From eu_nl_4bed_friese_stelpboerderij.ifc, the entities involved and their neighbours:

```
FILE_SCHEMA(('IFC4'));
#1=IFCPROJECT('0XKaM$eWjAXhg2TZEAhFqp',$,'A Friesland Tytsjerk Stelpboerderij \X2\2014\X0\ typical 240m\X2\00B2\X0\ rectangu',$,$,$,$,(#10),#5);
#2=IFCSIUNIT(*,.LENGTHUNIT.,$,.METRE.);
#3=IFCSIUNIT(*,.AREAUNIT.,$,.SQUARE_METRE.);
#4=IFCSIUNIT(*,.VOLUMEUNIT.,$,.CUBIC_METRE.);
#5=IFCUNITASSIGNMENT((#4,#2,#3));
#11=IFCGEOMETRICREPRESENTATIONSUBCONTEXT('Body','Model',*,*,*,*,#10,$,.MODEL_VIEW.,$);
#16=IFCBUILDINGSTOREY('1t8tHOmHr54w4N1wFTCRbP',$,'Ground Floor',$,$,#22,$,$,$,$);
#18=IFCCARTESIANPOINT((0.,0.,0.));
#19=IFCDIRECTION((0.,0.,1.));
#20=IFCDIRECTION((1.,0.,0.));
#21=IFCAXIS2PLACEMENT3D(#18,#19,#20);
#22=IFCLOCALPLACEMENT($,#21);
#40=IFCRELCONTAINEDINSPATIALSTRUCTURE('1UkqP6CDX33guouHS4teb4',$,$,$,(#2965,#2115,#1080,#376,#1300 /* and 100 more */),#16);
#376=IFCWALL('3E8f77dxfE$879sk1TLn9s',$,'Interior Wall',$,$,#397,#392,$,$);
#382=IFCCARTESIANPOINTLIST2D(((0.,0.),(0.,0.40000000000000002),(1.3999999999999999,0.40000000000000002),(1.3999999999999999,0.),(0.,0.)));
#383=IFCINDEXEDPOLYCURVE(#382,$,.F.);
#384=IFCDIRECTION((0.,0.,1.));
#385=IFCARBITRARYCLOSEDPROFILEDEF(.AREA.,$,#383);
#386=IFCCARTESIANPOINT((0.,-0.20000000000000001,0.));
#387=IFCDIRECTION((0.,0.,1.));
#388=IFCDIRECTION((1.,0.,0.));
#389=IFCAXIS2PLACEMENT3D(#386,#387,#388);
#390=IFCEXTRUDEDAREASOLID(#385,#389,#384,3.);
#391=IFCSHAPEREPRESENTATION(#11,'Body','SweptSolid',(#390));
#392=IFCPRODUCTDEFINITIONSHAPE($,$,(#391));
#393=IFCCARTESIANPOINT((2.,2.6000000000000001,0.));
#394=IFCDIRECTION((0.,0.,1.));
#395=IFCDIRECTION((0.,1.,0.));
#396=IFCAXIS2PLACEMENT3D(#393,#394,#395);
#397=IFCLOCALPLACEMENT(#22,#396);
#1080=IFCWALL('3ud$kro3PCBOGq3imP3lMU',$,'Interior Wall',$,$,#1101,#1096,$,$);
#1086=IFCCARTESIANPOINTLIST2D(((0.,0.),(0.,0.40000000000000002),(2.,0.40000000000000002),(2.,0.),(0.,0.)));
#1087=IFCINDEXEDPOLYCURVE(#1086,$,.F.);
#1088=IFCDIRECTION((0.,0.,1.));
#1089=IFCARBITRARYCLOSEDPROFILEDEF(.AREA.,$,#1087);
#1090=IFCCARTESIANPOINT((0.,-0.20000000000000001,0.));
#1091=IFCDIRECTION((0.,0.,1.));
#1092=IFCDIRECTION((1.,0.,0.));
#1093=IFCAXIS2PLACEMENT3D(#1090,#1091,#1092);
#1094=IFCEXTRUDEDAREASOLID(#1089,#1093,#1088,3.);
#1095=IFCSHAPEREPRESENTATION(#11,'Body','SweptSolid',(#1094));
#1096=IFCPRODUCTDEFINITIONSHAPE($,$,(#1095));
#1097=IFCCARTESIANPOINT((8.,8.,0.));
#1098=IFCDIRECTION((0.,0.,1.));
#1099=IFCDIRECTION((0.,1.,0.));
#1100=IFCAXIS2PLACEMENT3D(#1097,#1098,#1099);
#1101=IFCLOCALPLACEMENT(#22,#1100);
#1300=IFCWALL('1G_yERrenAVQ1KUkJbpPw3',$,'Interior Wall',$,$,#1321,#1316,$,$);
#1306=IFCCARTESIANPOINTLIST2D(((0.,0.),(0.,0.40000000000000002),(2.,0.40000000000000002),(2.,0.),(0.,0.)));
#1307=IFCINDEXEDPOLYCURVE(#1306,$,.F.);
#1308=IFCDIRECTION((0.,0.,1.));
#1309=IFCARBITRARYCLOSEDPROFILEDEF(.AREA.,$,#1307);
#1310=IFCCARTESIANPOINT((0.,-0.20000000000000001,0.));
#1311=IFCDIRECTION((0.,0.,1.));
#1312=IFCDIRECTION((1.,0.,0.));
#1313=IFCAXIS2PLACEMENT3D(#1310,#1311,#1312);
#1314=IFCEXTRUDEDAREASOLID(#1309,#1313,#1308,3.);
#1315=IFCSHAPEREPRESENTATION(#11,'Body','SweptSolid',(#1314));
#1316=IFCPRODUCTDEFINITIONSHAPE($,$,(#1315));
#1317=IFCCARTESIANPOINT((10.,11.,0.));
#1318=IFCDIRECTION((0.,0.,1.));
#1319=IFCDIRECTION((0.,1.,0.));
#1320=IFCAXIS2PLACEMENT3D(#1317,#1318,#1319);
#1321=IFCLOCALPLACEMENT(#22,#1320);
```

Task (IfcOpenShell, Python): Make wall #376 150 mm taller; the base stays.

```python
import ifcopenshell
import ifcopenshell.geom
import ifcopenshell.util.representation
import ifcopenshell.util.shape

model = ifcopenshell.open("eu_nl_4bed_friese_stelpboerderij.ifc")
settings = ifcopenshell.geom.settings()


def volume(element):
    """Net volume in cubic metres, openings subtracted."""
    shape = ifcopenshell.geom.create_shape(settings, element)
    return ifcopenshell.util.shape.get_volume(shape.geometry)


wall = model.by_id(376)
before = volume(wall)

body = ifcopenshell.util.representation.get_representation(wall, "Model", "Body")
solid = body.Items[0]
old_height = solid.Depth
solid.Depth += 0.15
after = volume(wall)

print(f"height {old_height:g} -> {solid.Depth:g}, volume {before:.3f} -> {after:.3f} m3")

model.write("eu_nl_4bed_friese_stelpboerderij-out.ifc")
```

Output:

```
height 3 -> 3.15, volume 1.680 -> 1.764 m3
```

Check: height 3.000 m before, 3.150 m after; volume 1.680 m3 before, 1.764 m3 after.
